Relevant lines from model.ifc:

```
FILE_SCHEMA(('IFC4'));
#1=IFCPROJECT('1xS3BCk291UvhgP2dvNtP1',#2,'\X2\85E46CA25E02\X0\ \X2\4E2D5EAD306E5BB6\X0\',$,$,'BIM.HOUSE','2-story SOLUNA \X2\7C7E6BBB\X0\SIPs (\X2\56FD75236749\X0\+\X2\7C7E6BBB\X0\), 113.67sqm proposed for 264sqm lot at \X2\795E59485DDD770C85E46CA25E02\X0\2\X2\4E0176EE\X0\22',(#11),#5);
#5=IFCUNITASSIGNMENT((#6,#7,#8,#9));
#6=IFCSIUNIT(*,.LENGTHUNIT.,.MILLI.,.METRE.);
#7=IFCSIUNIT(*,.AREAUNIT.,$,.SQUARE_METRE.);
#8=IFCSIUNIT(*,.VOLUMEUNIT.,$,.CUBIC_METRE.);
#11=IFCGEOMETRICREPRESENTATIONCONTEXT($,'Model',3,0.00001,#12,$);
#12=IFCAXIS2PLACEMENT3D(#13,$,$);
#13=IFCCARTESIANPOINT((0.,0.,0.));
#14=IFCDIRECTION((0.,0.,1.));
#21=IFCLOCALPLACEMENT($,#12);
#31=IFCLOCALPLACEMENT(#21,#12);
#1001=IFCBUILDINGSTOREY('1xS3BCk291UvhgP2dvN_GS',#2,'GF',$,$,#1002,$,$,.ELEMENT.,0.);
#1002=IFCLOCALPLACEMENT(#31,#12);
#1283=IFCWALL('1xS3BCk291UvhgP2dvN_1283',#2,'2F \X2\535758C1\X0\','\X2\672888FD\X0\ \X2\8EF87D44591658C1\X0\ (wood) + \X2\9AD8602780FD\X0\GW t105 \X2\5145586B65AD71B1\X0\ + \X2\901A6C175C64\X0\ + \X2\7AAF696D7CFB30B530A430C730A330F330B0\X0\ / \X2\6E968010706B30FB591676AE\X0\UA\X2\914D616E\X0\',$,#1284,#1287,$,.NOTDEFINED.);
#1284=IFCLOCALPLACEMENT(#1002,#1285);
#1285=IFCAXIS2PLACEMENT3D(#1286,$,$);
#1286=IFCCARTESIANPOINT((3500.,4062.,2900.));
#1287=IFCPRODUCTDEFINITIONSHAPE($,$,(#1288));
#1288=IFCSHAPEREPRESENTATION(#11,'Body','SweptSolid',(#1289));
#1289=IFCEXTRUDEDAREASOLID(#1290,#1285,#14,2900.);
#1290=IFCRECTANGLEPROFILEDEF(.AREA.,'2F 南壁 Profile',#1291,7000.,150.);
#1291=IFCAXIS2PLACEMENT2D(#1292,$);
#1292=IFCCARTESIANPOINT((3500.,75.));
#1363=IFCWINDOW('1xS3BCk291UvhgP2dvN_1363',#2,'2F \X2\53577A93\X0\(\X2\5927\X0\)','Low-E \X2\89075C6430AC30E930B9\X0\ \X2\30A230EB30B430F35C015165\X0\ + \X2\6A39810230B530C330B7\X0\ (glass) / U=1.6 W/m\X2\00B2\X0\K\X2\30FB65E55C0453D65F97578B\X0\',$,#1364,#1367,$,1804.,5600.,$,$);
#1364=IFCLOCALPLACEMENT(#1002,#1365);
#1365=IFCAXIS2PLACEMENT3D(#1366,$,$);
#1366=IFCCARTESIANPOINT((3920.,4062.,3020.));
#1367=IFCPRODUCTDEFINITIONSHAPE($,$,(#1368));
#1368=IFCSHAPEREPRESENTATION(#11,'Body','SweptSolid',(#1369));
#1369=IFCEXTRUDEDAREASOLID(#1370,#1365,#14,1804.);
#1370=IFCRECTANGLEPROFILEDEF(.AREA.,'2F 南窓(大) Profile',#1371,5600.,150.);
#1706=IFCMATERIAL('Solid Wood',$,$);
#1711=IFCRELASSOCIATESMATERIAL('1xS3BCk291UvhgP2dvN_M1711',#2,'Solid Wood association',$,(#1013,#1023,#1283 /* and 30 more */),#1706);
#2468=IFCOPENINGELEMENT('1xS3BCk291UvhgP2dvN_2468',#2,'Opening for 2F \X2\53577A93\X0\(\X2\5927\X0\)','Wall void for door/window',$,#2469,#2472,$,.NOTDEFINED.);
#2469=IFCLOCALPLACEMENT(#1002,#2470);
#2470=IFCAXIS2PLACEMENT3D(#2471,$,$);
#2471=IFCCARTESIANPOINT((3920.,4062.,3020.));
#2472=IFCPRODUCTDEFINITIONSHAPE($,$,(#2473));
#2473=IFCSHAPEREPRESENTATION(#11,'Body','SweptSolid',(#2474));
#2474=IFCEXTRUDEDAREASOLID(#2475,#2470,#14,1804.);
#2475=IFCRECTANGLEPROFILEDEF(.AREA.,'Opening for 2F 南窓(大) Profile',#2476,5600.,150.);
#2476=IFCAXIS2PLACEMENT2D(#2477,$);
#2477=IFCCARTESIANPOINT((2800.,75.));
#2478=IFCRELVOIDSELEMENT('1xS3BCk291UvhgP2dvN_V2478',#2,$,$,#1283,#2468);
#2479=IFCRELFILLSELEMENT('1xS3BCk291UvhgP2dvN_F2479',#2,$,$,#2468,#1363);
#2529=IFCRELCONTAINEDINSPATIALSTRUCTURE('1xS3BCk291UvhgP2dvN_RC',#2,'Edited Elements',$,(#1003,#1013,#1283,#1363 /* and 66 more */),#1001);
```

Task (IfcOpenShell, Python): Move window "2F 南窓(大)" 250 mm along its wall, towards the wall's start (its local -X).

```python
import ifcopenshell
import ifcopenshell.api.geometry
import ifcopenshell.util.placement

model = ifcopenshell.open("model.ifc")

window = model.by_id(1363)
opening = window.FillsVoids[0].RelatingOpeningElement
wall = opening.VoidsElements[0].RelatingBuildingElement

wall_matrix = ifcopenshell.util.placement.get_local_placement(wall.ObjectPlacement)
shift = wall_matrix[:3, 0] * -250.0
before = ifcopenshell.util.placement.get_local_placement(window.ObjectPlacement)[:3, 3].copy()

# The window is not placed relative to its opening, so move both.
for product in (opening, window):
    matrix = ifcopenshell.util.placement.get_local_placement(product.ObjectPlacement)
    matrix[:3, 3] += shift
    ifcopenshell.api.geometry.edit_object_placement(model, product=product, matrix=matrix, is_si=False)

after = ifcopenshell.util.placement.get_local_placement(window.ObjectPlacement)[:3, 3]
print("window moved by", (after - before).round(3) + 0.0)

model.write("model_edited.ifc")
```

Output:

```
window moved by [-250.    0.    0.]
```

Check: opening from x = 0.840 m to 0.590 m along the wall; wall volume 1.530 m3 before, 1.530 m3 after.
